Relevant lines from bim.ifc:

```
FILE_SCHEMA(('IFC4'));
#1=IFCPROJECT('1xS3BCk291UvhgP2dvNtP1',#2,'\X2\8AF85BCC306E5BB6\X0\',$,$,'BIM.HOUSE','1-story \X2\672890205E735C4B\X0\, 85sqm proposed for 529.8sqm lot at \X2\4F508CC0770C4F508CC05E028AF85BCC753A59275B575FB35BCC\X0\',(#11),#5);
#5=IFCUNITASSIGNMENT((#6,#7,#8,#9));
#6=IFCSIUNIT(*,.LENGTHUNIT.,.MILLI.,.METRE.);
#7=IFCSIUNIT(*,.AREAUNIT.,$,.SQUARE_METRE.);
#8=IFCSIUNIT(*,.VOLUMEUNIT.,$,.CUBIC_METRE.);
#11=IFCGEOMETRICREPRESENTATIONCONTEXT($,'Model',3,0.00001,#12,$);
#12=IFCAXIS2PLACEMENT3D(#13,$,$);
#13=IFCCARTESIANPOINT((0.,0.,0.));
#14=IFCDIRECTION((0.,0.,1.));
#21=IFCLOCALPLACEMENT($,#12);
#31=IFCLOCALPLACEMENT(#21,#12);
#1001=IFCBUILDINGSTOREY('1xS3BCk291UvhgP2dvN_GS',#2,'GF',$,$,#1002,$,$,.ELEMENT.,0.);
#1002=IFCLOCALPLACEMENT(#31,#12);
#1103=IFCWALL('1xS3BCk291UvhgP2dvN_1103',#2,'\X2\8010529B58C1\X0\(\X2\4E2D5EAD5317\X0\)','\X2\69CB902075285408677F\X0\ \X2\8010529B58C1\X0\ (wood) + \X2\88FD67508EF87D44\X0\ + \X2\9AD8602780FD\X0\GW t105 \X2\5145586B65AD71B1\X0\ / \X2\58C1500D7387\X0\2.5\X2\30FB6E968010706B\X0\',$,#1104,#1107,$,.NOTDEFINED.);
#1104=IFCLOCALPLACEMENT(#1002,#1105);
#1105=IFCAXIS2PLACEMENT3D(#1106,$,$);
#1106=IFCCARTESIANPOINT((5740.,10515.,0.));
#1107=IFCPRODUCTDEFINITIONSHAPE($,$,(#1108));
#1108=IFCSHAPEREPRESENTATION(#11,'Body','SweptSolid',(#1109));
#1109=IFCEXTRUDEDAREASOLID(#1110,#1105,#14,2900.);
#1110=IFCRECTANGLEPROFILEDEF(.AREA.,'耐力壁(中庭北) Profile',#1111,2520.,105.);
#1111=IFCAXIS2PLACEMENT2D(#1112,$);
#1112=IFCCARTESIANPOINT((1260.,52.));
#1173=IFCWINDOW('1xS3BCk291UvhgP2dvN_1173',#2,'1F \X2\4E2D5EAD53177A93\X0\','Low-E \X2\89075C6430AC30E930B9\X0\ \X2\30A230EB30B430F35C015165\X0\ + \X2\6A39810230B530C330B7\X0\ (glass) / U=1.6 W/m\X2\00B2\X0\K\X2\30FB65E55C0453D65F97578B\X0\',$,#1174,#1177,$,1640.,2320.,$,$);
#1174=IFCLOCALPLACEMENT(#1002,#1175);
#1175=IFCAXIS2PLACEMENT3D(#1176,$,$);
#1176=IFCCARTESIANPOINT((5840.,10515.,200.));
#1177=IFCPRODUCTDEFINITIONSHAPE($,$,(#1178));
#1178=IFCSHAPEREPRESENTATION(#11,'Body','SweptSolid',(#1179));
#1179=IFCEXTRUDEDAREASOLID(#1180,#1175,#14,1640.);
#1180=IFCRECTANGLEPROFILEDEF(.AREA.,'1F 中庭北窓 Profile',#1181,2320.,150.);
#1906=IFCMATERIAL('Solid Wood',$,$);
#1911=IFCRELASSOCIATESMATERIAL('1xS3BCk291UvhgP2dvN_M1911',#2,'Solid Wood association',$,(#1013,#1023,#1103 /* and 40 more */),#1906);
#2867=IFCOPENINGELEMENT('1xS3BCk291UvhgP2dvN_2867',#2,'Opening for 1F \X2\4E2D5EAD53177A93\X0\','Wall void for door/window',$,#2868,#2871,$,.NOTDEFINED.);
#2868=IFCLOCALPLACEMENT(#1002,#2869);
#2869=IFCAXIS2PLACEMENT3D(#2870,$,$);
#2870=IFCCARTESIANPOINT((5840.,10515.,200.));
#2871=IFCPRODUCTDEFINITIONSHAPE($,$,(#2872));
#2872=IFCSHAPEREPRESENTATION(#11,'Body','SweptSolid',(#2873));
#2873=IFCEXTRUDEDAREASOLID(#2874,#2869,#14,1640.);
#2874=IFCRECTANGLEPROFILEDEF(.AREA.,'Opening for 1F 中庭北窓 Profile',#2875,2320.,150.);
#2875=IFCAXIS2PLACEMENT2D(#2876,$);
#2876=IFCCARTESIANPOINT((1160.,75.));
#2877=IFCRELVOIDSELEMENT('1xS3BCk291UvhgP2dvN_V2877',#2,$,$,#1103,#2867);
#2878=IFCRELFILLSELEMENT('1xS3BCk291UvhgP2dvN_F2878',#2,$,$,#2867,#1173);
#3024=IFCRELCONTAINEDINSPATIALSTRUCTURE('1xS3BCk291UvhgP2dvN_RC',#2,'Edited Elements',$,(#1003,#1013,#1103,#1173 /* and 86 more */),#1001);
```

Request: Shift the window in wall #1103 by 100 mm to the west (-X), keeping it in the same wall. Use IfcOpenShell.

```python
import ifcopenshell
import ifcopenshell.api.geometry
import ifcopenshell.util.placement

model = ifcopenshell.open("bim.ifc")

window = model.by_id(1173)
opening = window.FillsVoids[0].RelatingOpeningElement
wall = opening.VoidsElements[0].RelatingBuildingElement

wall_matrix = ifcopenshell.util.placement.get_local_placement(wall.ObjectPlacement)
shift = wall_matrix[:3, 0] * -100.0
before = ifcopenshell.util.placement.get_local_placement(window.ObjectPlacement)[:3, 3].copy()

# The window is not placed relative to its opening, so move both.
for product in (opening, window):
    matrix = ifcopenshell.util.placement.get_local_placement(product.ObjectPlacement)
    matrix[:3, 3] += shift
    ifcopenshell.api.geometry.edit_object_placement(model, product=product, matrix=matrix, is_si=False)

after = ifcopenshell.util.placement.get_local_placement(window.ObjectPlacement)[:3, 3]
print("window moved by", (after - before).round(3) + 0.0)

model.write("bim_edited.ifc")
```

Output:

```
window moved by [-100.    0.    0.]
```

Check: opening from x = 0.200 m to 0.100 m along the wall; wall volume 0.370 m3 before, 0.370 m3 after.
